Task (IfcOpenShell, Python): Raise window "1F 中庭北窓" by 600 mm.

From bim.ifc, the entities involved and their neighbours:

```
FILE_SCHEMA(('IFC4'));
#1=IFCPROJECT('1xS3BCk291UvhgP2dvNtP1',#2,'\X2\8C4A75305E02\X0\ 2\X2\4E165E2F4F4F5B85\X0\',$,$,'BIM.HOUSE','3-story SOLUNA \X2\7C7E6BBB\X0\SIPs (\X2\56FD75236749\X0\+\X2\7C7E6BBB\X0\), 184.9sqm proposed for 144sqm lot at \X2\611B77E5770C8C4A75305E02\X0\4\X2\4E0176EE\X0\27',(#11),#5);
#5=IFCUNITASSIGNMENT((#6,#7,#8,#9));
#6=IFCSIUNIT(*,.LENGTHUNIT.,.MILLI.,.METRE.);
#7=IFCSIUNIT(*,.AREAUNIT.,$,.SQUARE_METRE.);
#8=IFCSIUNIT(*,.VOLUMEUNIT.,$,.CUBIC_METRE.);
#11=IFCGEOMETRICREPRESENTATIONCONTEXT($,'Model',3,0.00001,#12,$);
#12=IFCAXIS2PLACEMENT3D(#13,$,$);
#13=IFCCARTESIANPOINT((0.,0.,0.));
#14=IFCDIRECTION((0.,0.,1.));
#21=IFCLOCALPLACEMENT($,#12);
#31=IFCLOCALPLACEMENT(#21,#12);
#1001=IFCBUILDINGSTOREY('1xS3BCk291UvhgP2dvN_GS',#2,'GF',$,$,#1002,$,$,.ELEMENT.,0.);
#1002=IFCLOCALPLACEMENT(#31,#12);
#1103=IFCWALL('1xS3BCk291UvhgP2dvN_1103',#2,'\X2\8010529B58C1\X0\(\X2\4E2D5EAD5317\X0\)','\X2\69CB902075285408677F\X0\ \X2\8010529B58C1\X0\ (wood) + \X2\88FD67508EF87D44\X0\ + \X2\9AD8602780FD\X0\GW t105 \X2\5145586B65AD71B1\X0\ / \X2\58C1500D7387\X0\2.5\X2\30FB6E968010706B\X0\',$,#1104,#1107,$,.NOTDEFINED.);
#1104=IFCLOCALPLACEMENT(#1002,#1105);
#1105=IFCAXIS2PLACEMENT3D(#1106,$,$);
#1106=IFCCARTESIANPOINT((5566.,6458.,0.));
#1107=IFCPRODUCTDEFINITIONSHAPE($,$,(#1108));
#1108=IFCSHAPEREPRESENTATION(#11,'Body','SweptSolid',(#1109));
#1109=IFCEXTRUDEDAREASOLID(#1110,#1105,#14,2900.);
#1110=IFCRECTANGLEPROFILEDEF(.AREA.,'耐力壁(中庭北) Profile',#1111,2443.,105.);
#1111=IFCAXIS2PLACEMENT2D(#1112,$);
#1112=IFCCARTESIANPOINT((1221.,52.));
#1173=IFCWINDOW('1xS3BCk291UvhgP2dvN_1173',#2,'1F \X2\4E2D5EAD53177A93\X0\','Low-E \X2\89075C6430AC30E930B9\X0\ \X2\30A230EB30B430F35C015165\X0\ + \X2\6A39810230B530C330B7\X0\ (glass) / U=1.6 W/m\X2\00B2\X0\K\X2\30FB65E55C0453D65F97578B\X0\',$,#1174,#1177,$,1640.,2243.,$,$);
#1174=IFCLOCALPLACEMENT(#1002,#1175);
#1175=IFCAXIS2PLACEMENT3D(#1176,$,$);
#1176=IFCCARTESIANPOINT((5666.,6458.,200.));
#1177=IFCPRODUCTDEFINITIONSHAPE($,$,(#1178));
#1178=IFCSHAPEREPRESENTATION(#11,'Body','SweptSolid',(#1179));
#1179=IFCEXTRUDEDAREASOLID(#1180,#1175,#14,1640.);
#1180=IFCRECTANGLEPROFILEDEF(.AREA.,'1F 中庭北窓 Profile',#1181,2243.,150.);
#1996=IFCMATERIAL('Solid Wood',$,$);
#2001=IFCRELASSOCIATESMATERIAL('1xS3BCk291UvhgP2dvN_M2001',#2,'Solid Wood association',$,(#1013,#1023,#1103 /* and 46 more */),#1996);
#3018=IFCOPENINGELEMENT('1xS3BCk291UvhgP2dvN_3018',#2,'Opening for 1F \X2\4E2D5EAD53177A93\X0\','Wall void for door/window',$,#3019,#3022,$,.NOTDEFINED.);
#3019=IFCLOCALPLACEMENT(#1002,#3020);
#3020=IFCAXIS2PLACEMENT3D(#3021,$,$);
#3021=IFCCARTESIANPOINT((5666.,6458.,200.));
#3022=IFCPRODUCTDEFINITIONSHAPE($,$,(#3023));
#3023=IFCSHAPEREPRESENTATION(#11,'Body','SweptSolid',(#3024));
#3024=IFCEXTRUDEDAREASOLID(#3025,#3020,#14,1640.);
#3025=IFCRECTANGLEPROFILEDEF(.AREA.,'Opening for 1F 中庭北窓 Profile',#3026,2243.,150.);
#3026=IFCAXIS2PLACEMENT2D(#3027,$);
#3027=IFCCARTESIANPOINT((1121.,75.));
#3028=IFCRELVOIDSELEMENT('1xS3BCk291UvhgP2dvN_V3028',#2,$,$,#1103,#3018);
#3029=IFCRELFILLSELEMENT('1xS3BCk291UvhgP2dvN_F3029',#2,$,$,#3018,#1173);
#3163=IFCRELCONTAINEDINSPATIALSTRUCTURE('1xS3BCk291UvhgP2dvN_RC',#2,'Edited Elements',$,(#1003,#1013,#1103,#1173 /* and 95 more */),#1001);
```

```python
import numpy as np
import ifcopenshell
import ifcopenshell.api.geometry
import ifcopenshell.util.placement
import ifcopenshell.util.unit

model = ifcopenshell.open("bim.ifc")
unit_scale = ifcopenshell.util.unit.calculate_unit_scale(model)

window = model.by_id(1173)
opening = window.FillsVoids[0].RelatingOpeningElement
dz = 0.6 / unit_scale

shift = np.array([0.0, 0.0, dz])
# The window is not placed relative to its opening, so move both.
for product in (opening, window):
    matrix = ifcopenshell.util.placement.get_local_placement(product.ObjectPlacement)
    matrix[:3, 3] += shift
    ifcopenshell.api.geometry.edit_object_placement(model, product=product, matrix=matrix, is_si=False)

print(f"moved by {dz * unit_scale:+.3f} m")

model.write("bim_v2.ifc")
```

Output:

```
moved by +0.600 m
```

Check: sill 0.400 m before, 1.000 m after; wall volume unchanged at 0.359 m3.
